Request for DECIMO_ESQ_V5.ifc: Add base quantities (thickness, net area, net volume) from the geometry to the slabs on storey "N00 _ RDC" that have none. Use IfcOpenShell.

First a look at what the model holds.

```python
import ifcopenshell
import ifcopenshell.util.element
import ifcopenshell.util.unit

model = ifcopenshell.open("DECIMO_ESQ_V5.ifc")
print(model.schema)
for unit_type in ("LENGTHUNIT", "AREAUNIT", "VOLUMEUNIT"):
    print(unit_type, ifcopenshell.util.unit.calculate_unit_scale(model, unit_type))
storey = next(s for s in model.by_type("IfcBuildingStorey") if s.Name == "N00 _ RDC")
slabs = [e for e in ifcopenshell.util.element.get_decomposition(storey) if e.is_a("IfcSlab")]
for e in sorted(slabs, key=lambda e: e.id()):
    print(e.id(), e.is_a(), e.Name, list(ifcopenshell.util.element.get_psets(e, qtos_only=True)), sep=" | ")
```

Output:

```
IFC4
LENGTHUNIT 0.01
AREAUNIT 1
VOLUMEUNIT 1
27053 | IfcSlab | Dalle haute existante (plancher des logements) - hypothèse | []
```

```python
import ifcopenshell
import ifcopenshell.api.pset
import ifcopenshell.geom
import ifcopenshell.util.element
import ifcopenshell.util.shape
import ifcopenshell.util.unit

model = ifcopenshell.open("DECIMO_ESQ_V5.ifc")
unit_scale = ifcopenshell.util.unit.calculate_unit_scale(model)
area_scale = ifcopenshell.util.unit.calculate_unit_scale(model, "AREAUNIT")
volume_scale = ifcopenshell.util.unit.calculate_unit_scale(model, "VOLUMEUNIT")
settings = ifcopenshell.geom.settings()

storey = next(s for s in model.by_type("IfcBuildingStorey") if s.Name == "N00 _ RDC")
slabs = [e for e in ifcopenshell.util.element.get_decomposition(storey) if e.is_a("IfcSlab")]

for e in sorted(slabs, key=lambda e: e.id()):
    if ifcopenshell.util.element.get_psets(e, qtos_only=True, should_inherit=False):
        continue
    # Geometry comes back in metres, in the element's own axes.
    shape = ifcopenshell.geom.create_shape(settings, e)
    values = {
        "Width": ifcopenshell.util.shape.get_z(shape.geometry) / unit_scale,
        "NetArea": ifcopenshell.util.shape.get_footprint_area(shape.geometry) / area_scale,
        "NetVolume": ifcopenshell.util.shape.get_volume(shape.geometry) / volume_scale,
    }
    qto = ifcopenshell.api.pset.add_qto(model, product=e, name="Qto_SlabBaseQuantities")
    ifcopenshell.api.pset.edit_qto(model, qto=qto, properties=values)
    print(e.id(), {k: round(v, 3) for k, v in values.items()})

model.write("DECIMO_ESQ_V5-out.ifc")
```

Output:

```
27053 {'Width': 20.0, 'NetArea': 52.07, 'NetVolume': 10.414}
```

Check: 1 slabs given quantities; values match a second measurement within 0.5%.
